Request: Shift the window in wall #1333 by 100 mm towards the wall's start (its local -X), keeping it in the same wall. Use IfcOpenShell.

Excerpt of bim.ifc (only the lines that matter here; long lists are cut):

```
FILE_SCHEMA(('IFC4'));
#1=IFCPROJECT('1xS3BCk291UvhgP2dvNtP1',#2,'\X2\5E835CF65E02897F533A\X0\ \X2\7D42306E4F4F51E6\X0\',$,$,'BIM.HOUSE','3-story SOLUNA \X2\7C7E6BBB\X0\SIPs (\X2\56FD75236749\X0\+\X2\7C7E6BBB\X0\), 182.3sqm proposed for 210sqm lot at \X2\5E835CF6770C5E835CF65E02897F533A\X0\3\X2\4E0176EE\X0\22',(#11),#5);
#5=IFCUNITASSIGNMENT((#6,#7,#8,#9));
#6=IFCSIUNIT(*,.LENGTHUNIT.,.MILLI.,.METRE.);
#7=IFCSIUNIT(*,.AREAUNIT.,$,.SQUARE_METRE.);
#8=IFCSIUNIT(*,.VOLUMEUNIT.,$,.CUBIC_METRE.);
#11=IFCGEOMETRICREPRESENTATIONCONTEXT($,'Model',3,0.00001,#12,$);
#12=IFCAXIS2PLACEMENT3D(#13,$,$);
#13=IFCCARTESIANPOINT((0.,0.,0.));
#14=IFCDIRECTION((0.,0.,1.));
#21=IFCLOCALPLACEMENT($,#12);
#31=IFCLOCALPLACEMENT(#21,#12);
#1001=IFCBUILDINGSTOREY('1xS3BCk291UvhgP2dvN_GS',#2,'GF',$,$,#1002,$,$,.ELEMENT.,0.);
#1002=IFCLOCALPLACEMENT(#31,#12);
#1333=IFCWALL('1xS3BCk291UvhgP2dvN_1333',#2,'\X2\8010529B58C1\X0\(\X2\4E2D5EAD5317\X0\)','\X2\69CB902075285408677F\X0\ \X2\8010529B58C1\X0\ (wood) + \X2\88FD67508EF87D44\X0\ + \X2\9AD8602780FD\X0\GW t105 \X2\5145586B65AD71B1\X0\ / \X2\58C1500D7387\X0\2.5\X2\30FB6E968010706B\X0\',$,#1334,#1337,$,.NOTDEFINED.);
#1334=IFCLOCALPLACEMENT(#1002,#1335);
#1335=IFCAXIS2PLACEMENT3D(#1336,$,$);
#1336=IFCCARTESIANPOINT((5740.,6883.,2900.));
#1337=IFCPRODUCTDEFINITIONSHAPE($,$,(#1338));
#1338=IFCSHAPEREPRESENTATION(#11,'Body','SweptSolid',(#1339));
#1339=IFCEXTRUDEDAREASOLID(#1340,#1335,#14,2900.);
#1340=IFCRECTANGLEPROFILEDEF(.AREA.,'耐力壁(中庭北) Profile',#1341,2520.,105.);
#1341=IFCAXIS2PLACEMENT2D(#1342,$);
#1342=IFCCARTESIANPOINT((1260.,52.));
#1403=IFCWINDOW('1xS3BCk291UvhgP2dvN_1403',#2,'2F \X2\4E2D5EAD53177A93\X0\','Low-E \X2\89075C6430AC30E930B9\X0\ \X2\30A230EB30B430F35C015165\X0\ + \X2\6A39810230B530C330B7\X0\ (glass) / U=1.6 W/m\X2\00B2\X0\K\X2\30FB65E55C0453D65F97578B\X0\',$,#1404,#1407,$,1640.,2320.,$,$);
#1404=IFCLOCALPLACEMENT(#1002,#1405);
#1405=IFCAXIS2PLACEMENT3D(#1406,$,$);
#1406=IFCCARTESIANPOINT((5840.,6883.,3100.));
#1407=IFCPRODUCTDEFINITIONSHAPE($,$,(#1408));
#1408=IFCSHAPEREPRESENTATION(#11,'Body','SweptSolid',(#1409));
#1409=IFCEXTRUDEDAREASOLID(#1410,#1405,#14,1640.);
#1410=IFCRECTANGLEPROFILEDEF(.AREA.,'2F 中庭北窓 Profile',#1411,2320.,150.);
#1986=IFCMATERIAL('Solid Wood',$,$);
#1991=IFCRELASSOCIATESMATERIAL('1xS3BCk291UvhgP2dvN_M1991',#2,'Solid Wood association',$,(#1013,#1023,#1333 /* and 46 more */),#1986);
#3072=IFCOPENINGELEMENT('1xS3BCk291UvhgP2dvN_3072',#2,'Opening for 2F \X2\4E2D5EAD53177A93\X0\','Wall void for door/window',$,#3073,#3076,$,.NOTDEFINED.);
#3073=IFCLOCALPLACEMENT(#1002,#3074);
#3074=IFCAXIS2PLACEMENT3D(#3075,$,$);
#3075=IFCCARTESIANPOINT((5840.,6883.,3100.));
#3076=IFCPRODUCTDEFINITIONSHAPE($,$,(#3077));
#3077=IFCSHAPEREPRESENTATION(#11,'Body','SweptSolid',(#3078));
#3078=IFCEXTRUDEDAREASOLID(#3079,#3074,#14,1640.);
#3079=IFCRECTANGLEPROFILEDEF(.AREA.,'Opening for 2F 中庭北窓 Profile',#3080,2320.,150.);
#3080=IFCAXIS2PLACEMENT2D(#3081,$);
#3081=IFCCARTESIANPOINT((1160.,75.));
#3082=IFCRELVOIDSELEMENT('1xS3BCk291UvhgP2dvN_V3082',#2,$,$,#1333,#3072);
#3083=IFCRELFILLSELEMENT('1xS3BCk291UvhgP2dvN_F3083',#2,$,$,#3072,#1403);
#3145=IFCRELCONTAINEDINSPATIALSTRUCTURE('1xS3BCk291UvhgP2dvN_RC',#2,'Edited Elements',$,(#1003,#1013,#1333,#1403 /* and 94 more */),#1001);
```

```python
import ifcopenshell
import ifcopenshell.api.geometry
import ifcopenshell.util.placement
import ifcopenshell.util.unit

model = ifcopenshell.open("bim.ifc")
unit_scale = ifcopenshell.util.unit.calculate_unit_scale(model)

window = model.by_guid("1xS3BCk291UvhgP2dvN_1403")
opening = window.FillsVoids[0].RelatingOpeningElement
wall = opening.VoidsElements[0].RelatingBuildingElement

wall_matrix = ifcopenshell.util.placement.get_local_placement(wall.ObjectPlacement)
shift = wall_matrix[:3, 0] * -0.1 / unit_scale
before = ifcopenshell.util.placement.get_local_placement(window.ObjectPlacement)[:3, 3].copy()

# The window is not placed relative to its opening, so move both.
for product in (opening, window):
    matrix = ifcopenshell.util.placement.get_local_placement(product.ObjectPlacement)
    matrix[:3, 3] += shift
    ifcopenshell.api.geometry.edit_object_placement(model, product=product, matrix=matrix, is_si=False)

after = ifcopenshell.util.placement.get_local_placement(window.ObjectPlacement)[:3, 3]
print("window moved by", (after - before).round(3) + 0.0)

model.write("bim_v2.ifc")
```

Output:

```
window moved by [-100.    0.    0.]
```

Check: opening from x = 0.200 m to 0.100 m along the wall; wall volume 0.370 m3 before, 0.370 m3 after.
